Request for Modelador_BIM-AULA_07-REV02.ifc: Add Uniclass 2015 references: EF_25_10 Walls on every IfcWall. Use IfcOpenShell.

First a look at what the model holds.

```python
import ifcopenshell

model = ifcopenshell.open("Modelador_BIM-AULA_07-REV02.ifc")
print(model.schema)
print("classifications:", [c.Name for c in model.by_type("IfcClassification")])
for ifc_class in ("IfcDoor", "IfcRoof", "IfcStair", "IfcWall", "IfcWindow"):
    print(ifc_class, len(model.by_type(ifc_class)))
```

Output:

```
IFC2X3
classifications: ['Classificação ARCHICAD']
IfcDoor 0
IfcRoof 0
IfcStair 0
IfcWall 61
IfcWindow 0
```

```python
import ifcopenshell
import ifcopenshell.api.classification

model = ifcopenshell.open("Modelador_BIM-AULA_07-REV02.ifc")

# IFC2X3 requires Source and Edition and has no link from the project to the system.
system = model.create_entity("IfcClassification", Source="NBS", Edition="2015", Name="Uniclass 2015")

codes = {
    "IfcWall": ("EF_25_10", "Walls"),
}
for ifc_class, (code, name) in codes.items():
    products = model.by_type(ifc_class)
    ifcopenshell.api.classification.add_reference(
        model, products=products, classification=system, identification=code, name=name
    )
    print(code, len(products))

model.write("Modelador_BIM-AULA_07-REV02_updated.ifc")
```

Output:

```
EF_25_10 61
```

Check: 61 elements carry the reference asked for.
